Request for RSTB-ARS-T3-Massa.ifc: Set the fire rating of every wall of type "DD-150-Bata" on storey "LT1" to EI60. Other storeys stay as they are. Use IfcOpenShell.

First a look at what the model holds.

```python
import ifcopenshell
import ifcopenshell.util.element

model = ifcopenshell.open("RSTB-ARS-T3-Massa.ifc")
print(model.schema)
storey = next(s for s in model.by_type("IfcBuildingStorey") if s.Name == "LT1")
walls = [e for e in ifcopenshell.util.element.get_decomposition(storey) if e.is_a("IfcWall")]
seen = {}
for e in walls:
    element_type = ifcopenshell.util.element.get_type(e)
    key = (element_type.Name if element_type != e and element_type else None, ifcopenshell.util.element.get_pset(e, "Pset_WallCommon", "FireRating"))
    seen[key] = seen.get(key, 0) + 1
for (name, value), count in sorted(seen.items(), key=str):
    print(count, "x", name, "|", value)
```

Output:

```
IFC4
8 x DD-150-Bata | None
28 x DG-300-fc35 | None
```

```python
import ifcopenshell
import ifcopenshell.api.pset
import ifcopenshell.util.element

model = ifcopenshell.open("RSTB-ARS-T3-Massa.ifc")

storey = next(s for s in model.by_type("IfcBuildingStorey") if s.Name == "LT1")
walls = [e for e in ifcopenshell.util.element.get_decomposition(storey) if e.is_a("IfcWall")]

count = 0
for e in walls:
    element_type = ifcopenshell.util.element.get_type(e)
    if element_type in (None, e) or element_type.Name != "DD-150-Bata":
        continue
    # add_pset returns the element's existing set when there is one.
    pset = ifcopenshell.api.pset.add_pset(model, product=e, name="Pset_WallCommon")
    ifcopenshell.api.pset.edit_pset(model, pset=pset, properties={"FireRating": "EI60"})
    count += 1

print(count, "walls updated")

model.write("RSTB-ARS-T3-Massa_edited.ifc")
```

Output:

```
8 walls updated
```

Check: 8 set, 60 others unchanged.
